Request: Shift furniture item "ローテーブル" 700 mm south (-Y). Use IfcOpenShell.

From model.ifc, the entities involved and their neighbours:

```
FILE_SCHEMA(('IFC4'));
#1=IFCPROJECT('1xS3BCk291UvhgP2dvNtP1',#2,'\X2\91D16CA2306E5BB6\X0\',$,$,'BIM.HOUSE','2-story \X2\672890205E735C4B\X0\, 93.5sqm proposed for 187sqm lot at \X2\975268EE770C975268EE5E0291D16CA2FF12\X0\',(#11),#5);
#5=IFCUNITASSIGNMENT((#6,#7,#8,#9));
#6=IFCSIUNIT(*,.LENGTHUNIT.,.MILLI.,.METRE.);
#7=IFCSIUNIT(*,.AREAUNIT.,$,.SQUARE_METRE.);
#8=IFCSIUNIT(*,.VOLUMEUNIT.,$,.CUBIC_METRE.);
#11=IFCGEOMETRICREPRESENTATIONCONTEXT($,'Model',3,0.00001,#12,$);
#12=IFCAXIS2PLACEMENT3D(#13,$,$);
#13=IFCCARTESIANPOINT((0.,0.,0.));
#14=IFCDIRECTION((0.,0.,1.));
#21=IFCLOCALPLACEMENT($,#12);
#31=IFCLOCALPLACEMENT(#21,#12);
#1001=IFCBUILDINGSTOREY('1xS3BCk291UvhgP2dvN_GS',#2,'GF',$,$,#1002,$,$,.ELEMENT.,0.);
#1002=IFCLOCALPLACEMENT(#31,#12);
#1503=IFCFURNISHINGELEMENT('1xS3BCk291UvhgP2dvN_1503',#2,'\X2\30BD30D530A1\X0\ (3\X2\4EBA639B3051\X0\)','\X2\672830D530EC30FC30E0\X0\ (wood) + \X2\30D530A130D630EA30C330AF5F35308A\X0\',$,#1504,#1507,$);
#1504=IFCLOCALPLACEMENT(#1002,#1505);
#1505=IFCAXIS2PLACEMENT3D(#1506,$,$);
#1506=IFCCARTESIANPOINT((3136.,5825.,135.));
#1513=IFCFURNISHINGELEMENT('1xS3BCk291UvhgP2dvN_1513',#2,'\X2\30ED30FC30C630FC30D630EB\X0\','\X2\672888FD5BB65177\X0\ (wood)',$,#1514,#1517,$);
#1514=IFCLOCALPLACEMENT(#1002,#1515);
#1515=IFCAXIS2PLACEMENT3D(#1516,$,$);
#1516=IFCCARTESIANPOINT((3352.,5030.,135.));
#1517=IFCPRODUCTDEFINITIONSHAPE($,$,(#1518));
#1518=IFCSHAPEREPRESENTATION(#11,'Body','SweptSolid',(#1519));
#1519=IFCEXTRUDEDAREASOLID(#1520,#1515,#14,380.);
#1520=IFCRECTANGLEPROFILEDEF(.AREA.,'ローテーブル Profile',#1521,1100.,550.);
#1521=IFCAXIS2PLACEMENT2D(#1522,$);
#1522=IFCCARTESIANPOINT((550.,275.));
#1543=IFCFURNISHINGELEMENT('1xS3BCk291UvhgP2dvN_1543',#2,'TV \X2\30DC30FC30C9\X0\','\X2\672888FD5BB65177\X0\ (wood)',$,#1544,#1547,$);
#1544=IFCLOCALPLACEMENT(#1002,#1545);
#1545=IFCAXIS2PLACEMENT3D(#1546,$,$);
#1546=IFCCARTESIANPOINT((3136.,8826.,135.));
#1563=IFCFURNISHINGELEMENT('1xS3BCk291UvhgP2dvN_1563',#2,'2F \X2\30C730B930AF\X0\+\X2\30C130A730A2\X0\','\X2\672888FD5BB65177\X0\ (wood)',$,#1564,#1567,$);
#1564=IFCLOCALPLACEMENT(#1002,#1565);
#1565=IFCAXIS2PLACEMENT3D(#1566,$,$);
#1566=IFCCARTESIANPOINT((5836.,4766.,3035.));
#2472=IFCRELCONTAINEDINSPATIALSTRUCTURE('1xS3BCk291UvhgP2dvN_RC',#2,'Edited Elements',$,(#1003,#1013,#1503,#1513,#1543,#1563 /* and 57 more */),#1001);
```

```python
import ifcopenshell
import ifcopenshell.api.geometry
import ifcopenshell.util.placement
import ifcopenshell.util.unit

model = ifcopenshell.open("model.ifc")
unit_scale = ifcopenshell.util.unit.calculate_unit_scale(model)

item = model.by_id(1513)
matrix = ifcopenshell.util.placement.get_local_placement(item.ObjectPlacement)
matrix[1, 3] -= 0.7 / unit_scale
ifcopenshell.api.geometry.edit_object_placement(model, product=item, matrix=matrix, is_si=False)

print(ifcopenshell.util.placement.get_local_placement(item.ObjectPlacement).round(3) + 0.0)

model.write("model_rev.ifc")
```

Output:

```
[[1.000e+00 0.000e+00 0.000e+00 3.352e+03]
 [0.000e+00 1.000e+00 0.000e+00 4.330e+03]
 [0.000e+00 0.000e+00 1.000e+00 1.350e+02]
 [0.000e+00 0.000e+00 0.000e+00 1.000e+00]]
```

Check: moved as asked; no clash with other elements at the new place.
